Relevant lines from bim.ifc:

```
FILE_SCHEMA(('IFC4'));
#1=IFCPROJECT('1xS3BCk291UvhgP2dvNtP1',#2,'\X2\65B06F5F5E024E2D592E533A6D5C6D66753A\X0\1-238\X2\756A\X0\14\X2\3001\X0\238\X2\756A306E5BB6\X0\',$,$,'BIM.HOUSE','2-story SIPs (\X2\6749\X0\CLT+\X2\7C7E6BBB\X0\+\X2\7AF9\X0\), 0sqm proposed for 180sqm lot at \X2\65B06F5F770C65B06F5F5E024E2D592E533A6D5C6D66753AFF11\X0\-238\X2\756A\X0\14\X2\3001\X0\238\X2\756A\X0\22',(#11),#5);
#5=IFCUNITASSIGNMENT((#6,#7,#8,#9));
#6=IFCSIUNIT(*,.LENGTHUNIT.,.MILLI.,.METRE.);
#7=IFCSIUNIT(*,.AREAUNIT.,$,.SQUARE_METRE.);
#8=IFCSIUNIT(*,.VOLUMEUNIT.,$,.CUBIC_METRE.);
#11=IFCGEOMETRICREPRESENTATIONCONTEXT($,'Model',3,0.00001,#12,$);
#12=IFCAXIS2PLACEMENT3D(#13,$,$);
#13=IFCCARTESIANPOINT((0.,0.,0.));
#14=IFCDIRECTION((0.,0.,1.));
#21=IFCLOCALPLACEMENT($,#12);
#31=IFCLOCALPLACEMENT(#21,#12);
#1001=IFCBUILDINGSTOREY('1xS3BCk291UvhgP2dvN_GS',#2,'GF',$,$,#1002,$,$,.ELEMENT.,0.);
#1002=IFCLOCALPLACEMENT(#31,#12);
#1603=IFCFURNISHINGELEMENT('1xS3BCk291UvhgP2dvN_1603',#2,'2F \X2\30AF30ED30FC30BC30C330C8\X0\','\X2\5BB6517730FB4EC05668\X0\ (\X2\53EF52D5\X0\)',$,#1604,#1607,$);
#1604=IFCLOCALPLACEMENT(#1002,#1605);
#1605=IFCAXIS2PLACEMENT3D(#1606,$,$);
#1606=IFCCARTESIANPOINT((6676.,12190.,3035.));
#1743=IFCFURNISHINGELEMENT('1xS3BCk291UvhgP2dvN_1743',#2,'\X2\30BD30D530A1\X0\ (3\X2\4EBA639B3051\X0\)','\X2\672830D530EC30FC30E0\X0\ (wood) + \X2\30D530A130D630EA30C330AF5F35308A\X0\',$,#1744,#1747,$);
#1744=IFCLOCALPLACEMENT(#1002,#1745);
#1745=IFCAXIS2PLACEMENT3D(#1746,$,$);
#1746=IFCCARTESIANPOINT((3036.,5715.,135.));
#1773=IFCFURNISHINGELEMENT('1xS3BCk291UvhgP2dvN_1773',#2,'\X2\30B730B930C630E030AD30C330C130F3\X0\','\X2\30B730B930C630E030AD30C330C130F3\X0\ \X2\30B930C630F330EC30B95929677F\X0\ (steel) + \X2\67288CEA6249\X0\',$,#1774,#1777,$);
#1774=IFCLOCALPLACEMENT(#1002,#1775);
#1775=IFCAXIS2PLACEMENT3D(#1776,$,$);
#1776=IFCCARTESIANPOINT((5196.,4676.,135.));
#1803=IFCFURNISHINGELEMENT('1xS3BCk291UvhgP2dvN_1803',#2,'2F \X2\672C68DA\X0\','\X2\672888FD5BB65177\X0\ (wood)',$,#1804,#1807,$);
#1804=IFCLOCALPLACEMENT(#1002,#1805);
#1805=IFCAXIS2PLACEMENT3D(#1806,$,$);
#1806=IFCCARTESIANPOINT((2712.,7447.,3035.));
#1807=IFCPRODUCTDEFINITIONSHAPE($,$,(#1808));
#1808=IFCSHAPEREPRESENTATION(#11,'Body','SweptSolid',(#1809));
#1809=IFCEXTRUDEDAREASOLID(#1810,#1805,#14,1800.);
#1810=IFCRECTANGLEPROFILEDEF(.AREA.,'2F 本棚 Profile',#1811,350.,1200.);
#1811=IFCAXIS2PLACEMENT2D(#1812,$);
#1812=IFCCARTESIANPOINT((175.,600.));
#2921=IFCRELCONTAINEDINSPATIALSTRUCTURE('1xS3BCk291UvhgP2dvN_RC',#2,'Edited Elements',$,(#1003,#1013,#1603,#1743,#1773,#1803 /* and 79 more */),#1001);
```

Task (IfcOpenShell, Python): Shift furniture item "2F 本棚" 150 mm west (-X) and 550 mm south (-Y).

```python
import ifcopenshell
import ifcopenshell.api.geometry
import ifcopenshell.util.placement

model = ifcopenshell.open("bim.ifc")

item = model.by_guid("1xS3BCk291UvhgP2dvN_1803")
matrix = ifcopenshell.util.placement.get_local_placement(item.ObjectPlacement)
matrix[0, 3] -= 150.0
matrix[1, 3] -= 550.0
ifcopenshell.api.geometry.edit_object_placement(model, product=item, matrix=matrix, is_si=False)

print(ifcopenshell.util.placement.get_local_placement(item.ObjectPlacement).round(3) + 0.0)

model.write("bim_edited.ifc")
```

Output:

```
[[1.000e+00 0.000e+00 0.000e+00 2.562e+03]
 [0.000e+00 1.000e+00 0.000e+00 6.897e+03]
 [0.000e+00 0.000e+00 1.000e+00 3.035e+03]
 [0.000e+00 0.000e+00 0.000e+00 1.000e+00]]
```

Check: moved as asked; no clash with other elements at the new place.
